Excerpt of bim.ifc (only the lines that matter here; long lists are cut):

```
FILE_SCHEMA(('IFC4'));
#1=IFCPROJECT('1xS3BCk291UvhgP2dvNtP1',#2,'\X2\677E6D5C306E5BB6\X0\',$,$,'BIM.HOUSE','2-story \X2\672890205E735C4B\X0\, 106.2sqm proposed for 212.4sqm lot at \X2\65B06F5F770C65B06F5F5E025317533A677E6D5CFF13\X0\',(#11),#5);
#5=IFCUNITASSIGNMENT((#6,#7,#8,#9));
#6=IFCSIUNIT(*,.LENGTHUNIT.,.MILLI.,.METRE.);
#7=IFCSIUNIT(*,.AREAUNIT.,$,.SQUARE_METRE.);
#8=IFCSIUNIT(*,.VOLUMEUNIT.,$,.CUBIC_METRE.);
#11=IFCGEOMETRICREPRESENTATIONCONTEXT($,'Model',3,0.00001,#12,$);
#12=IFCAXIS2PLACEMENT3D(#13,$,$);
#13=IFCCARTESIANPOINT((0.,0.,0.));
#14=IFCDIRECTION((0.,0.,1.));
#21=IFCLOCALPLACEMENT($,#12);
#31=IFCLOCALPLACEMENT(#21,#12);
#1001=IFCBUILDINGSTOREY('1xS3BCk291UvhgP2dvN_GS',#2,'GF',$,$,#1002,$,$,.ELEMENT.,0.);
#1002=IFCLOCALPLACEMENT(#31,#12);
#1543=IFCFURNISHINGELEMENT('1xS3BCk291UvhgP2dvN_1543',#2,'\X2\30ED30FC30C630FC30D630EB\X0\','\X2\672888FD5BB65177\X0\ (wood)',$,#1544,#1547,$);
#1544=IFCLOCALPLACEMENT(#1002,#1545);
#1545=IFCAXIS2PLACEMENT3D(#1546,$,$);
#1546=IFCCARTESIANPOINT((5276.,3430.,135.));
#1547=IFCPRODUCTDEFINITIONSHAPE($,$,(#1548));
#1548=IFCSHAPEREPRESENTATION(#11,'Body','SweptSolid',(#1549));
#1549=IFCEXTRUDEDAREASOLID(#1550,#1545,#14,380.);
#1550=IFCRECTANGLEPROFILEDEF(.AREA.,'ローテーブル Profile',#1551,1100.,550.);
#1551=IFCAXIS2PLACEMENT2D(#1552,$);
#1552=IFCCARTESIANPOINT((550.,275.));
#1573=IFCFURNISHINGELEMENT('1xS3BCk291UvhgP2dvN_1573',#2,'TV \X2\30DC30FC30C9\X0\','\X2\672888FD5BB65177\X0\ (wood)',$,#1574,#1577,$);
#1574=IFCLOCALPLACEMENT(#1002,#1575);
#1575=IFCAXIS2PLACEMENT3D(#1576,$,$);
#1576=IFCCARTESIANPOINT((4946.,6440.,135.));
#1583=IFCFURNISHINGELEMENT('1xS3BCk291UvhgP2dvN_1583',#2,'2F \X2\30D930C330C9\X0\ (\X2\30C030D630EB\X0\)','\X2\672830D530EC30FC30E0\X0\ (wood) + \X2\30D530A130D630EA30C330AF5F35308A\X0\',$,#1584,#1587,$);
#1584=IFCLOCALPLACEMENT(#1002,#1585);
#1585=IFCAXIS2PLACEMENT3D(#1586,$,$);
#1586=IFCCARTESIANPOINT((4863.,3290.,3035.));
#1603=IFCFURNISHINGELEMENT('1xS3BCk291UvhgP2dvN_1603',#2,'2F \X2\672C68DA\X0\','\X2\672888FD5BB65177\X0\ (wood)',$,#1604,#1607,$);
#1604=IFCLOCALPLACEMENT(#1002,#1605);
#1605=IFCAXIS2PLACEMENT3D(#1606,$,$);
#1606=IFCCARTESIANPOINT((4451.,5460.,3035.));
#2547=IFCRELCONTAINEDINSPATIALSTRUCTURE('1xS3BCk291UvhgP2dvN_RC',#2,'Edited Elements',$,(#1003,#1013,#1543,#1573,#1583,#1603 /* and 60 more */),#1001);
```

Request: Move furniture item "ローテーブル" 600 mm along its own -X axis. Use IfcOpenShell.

```python
import ifcopenshell
import ifcopenshell.api.geometry
import ifcopenshell.util.placement

model = ifcopenshell.open("bim.ifc")

item = model.by_guid("1xS3BCk291UvhgP2dvN_1543")
matrix = ifcopenshell.util.placement.get_local_placement(item.ObjectPlacement)
matrix[:3, 3] -= matrix[:3, 0] * 600.0
ifcopenshell.api.geometry.edit_object_placement(model, product=item, matrix=matrix, is_si=False)

print(ifcopenshell.util.placement.get_local_placement(item.ObjectPlacement).round(3) + 0.0)

model.write("bim_edited.ifc")
```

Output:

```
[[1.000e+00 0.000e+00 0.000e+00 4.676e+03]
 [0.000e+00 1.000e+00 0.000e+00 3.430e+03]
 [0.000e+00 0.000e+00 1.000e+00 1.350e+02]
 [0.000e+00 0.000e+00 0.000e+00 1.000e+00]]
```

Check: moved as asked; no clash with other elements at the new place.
